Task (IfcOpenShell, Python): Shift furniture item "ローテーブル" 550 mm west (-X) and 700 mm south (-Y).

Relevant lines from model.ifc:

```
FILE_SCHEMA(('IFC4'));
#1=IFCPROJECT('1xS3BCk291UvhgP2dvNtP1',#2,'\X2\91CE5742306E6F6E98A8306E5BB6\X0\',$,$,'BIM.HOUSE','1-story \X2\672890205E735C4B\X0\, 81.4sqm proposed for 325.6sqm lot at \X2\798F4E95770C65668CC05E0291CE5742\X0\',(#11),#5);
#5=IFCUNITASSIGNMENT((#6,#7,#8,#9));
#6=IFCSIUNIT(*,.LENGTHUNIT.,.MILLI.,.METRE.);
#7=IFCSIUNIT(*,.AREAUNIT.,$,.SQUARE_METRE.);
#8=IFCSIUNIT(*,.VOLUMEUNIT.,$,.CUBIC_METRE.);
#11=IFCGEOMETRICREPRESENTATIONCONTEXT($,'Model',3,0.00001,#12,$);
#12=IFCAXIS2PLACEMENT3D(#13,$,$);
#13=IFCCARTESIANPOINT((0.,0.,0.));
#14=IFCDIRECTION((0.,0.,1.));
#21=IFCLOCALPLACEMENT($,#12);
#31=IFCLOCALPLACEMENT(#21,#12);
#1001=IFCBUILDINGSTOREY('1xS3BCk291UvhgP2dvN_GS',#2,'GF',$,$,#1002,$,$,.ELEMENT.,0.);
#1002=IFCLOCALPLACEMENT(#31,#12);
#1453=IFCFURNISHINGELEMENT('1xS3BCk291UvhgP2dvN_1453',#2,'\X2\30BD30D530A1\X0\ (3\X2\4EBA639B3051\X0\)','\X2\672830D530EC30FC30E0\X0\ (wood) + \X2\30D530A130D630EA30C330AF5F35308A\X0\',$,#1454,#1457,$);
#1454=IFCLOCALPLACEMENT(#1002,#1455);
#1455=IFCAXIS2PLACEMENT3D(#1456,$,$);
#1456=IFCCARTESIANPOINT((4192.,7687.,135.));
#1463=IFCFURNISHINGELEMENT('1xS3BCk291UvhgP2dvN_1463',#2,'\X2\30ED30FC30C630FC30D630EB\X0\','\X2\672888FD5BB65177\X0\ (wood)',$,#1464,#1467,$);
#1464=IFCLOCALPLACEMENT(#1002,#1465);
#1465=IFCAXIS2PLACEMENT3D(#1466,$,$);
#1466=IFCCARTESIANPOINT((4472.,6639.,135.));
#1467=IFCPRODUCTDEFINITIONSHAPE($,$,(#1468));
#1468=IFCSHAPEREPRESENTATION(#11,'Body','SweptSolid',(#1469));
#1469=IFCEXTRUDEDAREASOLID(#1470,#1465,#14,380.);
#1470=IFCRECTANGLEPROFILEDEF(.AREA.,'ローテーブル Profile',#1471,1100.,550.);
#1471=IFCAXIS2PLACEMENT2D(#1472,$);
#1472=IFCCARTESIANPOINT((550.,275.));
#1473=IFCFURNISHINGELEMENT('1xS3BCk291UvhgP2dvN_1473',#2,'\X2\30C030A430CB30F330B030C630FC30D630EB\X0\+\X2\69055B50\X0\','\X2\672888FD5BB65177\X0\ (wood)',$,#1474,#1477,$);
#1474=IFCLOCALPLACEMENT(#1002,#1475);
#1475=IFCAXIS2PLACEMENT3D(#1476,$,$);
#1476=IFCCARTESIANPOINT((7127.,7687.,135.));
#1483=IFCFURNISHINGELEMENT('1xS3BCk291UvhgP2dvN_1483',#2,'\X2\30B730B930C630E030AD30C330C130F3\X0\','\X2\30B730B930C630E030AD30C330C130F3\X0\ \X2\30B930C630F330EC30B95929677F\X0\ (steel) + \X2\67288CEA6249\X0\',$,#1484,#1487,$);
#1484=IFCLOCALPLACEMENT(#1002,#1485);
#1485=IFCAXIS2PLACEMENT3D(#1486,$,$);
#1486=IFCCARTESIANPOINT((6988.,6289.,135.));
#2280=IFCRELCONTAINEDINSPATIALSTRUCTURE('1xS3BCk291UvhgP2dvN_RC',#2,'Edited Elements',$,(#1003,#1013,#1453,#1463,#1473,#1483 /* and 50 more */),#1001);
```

```python
import ifcopenshell
import ifcopenshell.api.geometry
import ifcopenshell.util.placement
import ifcopenshell.util.unit

model = ifcopenshell.open("model.ifc")
unit_scale = ifcopenshell.util.unit.calculate_unit_scale(model)

item = model.by_guid("1xS3BCk291UvhgP2dvN_1463")
matrix = ifcopenshell.util.placement.get_local_placement(item.ObjectPlacement)
matrix[0, 3] -= 0.55 / unit_scale
matrix[1, 3] -= 0.7 / unit_scale
ifcopenshell.api.geometry.edit_object_placement(model, product=item, matrix=matrix, is_si=False)

print(ifcopenshell.util.placement.get_local_placement(item.ObjectPlacement).round(3) + 0.0)

model.write("model_rev.ifc")
```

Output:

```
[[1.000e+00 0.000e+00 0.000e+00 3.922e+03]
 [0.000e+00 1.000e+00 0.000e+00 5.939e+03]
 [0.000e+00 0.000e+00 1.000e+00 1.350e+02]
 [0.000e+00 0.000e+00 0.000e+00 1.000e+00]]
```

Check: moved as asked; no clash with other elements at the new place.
